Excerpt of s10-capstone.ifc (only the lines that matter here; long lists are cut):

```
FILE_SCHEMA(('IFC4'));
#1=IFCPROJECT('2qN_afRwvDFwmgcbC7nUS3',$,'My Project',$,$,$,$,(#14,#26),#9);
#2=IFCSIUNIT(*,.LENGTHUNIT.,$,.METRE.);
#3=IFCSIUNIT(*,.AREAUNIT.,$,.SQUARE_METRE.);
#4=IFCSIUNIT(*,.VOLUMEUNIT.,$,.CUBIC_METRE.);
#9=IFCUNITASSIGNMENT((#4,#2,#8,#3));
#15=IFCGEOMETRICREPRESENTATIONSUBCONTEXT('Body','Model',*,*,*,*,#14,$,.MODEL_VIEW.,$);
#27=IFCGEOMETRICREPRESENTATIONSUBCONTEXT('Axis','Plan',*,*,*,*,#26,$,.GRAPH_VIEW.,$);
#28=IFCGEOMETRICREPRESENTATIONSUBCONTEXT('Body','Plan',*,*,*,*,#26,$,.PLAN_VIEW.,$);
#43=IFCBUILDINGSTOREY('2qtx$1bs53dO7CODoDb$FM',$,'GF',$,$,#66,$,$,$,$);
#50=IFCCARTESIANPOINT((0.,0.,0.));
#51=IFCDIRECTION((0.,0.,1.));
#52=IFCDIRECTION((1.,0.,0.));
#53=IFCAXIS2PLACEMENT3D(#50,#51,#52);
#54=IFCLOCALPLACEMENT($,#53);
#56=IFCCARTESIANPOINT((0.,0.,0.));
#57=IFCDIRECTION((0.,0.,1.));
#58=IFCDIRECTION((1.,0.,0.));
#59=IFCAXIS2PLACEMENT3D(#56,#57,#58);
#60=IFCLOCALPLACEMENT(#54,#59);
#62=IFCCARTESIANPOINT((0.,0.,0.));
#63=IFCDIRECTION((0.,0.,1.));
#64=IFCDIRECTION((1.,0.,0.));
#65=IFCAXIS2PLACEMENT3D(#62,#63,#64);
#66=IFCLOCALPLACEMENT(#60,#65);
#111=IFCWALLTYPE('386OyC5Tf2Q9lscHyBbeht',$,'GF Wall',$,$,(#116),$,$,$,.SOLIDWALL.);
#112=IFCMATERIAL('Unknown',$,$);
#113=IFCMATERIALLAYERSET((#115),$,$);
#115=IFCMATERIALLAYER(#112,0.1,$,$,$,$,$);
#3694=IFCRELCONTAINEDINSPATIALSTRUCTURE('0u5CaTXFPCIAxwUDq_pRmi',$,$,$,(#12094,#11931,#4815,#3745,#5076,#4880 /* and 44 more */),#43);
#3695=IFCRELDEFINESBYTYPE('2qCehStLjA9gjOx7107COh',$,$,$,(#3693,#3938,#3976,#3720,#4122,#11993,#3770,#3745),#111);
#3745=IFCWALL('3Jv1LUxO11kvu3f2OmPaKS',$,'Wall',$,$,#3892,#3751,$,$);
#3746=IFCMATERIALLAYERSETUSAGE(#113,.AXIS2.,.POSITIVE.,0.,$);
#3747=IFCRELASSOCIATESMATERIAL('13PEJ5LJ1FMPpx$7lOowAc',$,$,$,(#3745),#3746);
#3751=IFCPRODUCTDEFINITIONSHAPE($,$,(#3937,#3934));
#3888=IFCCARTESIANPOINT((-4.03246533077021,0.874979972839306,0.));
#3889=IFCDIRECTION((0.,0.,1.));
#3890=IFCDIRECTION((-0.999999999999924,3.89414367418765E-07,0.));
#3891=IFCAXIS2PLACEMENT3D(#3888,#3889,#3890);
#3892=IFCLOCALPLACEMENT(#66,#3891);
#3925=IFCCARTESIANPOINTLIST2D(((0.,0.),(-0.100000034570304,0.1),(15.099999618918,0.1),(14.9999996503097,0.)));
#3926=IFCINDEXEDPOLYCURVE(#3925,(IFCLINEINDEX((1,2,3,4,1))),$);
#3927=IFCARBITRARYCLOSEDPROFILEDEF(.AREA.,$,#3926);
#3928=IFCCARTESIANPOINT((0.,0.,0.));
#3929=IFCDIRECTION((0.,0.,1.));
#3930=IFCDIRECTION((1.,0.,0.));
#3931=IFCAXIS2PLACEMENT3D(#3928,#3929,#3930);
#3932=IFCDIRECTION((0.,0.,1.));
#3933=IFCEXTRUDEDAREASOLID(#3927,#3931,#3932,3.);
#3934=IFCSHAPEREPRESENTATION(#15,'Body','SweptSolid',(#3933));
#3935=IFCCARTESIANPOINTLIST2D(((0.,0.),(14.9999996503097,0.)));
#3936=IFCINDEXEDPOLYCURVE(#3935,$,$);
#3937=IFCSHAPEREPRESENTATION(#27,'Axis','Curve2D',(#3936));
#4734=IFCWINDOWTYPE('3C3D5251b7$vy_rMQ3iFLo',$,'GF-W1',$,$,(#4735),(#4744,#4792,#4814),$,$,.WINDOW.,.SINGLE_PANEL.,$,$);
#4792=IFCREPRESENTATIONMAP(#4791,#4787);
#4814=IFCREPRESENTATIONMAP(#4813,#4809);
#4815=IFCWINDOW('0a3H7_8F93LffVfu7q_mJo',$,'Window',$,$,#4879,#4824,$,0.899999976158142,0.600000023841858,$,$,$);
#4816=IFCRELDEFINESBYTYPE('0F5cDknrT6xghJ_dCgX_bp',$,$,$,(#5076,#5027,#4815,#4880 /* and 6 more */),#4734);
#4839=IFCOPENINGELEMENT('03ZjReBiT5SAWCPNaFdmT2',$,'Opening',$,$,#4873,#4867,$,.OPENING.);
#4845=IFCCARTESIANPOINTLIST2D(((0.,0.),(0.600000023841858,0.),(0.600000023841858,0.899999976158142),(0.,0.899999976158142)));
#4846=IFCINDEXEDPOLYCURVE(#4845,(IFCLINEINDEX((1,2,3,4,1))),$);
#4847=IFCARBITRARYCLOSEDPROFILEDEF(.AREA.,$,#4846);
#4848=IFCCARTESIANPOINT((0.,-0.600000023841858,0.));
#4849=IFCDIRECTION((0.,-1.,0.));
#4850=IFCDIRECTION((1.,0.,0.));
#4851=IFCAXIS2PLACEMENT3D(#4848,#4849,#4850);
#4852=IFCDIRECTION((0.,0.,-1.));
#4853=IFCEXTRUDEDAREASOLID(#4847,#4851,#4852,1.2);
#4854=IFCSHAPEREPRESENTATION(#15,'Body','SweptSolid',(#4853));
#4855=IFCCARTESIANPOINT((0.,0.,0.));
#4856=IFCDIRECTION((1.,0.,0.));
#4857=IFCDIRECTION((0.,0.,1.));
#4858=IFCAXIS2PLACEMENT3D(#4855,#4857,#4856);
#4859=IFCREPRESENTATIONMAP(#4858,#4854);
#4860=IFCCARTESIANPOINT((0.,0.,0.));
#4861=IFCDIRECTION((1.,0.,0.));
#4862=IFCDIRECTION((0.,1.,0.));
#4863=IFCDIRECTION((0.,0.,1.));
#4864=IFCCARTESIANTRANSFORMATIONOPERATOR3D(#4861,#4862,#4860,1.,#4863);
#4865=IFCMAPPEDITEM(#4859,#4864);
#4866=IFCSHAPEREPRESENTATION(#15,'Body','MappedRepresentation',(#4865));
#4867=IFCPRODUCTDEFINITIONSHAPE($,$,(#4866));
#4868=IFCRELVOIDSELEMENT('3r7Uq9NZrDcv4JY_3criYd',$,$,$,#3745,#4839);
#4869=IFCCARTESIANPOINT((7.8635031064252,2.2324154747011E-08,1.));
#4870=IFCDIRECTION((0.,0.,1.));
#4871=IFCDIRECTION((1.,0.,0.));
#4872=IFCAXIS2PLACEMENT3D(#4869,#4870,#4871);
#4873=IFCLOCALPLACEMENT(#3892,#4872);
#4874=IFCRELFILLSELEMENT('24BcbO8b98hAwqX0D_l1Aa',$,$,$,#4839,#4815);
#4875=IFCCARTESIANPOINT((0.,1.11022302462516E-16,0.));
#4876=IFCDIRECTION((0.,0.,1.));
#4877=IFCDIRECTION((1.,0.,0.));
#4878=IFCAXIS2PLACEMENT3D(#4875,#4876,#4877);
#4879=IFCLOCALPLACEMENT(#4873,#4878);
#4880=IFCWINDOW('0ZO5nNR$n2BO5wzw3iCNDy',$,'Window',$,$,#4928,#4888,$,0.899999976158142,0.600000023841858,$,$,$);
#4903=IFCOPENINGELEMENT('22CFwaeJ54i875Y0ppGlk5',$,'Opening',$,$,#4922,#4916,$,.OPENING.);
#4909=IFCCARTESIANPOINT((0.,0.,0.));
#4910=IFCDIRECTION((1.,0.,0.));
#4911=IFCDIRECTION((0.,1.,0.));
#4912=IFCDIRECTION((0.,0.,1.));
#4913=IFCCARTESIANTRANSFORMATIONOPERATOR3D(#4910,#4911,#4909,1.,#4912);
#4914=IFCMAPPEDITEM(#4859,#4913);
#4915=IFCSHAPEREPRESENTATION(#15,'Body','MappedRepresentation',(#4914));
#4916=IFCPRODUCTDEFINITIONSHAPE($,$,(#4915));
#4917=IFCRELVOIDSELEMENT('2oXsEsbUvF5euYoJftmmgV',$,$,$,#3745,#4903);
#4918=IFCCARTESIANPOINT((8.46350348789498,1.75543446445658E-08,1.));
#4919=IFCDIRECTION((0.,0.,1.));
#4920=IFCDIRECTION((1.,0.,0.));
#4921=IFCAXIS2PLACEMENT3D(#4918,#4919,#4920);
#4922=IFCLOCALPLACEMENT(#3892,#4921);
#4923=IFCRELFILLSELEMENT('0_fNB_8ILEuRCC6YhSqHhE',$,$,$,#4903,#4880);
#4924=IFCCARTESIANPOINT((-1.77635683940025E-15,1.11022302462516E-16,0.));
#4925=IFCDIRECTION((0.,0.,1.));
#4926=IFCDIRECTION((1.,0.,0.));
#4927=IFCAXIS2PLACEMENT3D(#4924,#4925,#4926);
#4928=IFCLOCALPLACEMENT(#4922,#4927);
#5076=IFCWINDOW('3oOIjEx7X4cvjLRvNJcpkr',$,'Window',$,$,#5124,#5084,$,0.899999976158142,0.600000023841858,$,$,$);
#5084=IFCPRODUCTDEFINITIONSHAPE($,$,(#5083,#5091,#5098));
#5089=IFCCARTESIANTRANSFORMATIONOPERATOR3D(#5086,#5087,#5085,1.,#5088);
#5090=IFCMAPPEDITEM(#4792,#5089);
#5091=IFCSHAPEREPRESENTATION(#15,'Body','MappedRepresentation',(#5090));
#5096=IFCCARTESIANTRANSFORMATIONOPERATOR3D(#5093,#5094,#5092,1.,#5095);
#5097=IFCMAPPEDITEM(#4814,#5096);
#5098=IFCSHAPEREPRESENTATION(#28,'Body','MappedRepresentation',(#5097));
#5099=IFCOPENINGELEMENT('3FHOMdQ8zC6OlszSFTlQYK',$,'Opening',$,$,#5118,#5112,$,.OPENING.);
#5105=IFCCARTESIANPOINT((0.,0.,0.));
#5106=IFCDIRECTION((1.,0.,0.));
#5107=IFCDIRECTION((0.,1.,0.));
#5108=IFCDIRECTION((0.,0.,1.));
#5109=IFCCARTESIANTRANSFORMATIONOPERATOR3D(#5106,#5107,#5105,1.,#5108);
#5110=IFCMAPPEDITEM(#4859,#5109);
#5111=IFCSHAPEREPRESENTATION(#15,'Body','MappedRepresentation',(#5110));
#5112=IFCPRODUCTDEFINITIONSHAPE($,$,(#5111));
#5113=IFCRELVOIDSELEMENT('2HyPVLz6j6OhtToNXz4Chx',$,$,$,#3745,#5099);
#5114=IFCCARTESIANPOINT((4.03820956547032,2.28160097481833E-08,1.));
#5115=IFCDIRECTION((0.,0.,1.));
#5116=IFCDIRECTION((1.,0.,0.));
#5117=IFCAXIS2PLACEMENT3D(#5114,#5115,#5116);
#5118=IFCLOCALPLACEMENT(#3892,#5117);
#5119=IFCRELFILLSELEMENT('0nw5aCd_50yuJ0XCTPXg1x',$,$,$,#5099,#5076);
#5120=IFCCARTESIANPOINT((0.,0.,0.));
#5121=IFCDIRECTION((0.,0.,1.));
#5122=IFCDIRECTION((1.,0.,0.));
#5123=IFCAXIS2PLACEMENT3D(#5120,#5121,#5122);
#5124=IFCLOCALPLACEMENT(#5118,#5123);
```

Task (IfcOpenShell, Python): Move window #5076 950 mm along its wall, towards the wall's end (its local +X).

```python
import ifcopenshell
import ifcopenshell.api.geometry
import ifcopenshell.util.placement

model = ifcopenshell.open("s10-capstone.ifc")

window = model.by_guid("3oOIjEx7X4cvjLRvNJcpkr")
opening = window.FillsVoids[0].RelatingOpeningElement
wall = opening.VoidsElements[0].RelatingBuildingElement

wall_matrix = ifcopenshell.util.placement.get_local_placement(wall.ObjectPlacement)
shift = wall_matrix[:3, 0] * 0.95
before = ifcopenshell.util.placement.get_local_placement(window.ObjectPlacement)[:3, 3].copy()

# The window is placed relative to its opening, so it follows when the opening moves.
matrix = ifcopenshell.util.placement.get_local_placement(opening.ObjectPlacement)
matrix[:3, 3] += shift
ifcopenshell.api.geometry.edit_object_placement(
    model, product=opening, matrix=matrix, is_si=False, should_transform_children=True
)

after = ifcopenshell.util.placement.get_local_placement(window.ObjectPlacement)[:3, 3]
print("window moved by", (after - before).round(3) + 0.0)

model.write("s10-capstone_rev.ifc")
```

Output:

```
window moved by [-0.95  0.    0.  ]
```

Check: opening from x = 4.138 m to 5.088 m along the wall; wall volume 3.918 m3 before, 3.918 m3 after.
